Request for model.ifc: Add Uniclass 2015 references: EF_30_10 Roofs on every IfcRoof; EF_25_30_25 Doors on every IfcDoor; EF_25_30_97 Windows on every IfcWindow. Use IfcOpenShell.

First a look at what the model holds.

```python
import ifcopenshell

model = ifcopenshell.open("model.ifc")
print(model.schema)
print("classifications:", [c.Name for c in model.by_type("IfcClassification")])
for ifc_class in ("IfcDoor", "IfcRoof", "IfcStair", "IfcWall", "IfcWindow"):
    print(ifc_class, len(model.by_type(ifc_class)))
```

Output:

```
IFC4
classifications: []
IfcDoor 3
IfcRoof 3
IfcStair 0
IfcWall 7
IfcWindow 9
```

```python
import ifcopenshell
import ifcopenshell.api.classification

model = ifcopenshell.open("model.ifc")

system = ifcopenshell.api.classification.add_classification(model, classification="Uniclass 2015")

codes = {
    "IfcRoof": ("EF_30_10", "Roofs"),
    "IfcDoor": ("EF_25_30_25", "Doors"),
    "IfcWindow": ("EF_25_30_97", "Windows"),
}
for ifc_class, (code, name) in codes.items():
    products = model.by_type(ifc_class)
    ifcopenshell.api.classification.add_reference(
        model, products=products, classification=system, identification=code, name=name
    )
    print(code, len(products))

model.write("model_v2.ifc")
```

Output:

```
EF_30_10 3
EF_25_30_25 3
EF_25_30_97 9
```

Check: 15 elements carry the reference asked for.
